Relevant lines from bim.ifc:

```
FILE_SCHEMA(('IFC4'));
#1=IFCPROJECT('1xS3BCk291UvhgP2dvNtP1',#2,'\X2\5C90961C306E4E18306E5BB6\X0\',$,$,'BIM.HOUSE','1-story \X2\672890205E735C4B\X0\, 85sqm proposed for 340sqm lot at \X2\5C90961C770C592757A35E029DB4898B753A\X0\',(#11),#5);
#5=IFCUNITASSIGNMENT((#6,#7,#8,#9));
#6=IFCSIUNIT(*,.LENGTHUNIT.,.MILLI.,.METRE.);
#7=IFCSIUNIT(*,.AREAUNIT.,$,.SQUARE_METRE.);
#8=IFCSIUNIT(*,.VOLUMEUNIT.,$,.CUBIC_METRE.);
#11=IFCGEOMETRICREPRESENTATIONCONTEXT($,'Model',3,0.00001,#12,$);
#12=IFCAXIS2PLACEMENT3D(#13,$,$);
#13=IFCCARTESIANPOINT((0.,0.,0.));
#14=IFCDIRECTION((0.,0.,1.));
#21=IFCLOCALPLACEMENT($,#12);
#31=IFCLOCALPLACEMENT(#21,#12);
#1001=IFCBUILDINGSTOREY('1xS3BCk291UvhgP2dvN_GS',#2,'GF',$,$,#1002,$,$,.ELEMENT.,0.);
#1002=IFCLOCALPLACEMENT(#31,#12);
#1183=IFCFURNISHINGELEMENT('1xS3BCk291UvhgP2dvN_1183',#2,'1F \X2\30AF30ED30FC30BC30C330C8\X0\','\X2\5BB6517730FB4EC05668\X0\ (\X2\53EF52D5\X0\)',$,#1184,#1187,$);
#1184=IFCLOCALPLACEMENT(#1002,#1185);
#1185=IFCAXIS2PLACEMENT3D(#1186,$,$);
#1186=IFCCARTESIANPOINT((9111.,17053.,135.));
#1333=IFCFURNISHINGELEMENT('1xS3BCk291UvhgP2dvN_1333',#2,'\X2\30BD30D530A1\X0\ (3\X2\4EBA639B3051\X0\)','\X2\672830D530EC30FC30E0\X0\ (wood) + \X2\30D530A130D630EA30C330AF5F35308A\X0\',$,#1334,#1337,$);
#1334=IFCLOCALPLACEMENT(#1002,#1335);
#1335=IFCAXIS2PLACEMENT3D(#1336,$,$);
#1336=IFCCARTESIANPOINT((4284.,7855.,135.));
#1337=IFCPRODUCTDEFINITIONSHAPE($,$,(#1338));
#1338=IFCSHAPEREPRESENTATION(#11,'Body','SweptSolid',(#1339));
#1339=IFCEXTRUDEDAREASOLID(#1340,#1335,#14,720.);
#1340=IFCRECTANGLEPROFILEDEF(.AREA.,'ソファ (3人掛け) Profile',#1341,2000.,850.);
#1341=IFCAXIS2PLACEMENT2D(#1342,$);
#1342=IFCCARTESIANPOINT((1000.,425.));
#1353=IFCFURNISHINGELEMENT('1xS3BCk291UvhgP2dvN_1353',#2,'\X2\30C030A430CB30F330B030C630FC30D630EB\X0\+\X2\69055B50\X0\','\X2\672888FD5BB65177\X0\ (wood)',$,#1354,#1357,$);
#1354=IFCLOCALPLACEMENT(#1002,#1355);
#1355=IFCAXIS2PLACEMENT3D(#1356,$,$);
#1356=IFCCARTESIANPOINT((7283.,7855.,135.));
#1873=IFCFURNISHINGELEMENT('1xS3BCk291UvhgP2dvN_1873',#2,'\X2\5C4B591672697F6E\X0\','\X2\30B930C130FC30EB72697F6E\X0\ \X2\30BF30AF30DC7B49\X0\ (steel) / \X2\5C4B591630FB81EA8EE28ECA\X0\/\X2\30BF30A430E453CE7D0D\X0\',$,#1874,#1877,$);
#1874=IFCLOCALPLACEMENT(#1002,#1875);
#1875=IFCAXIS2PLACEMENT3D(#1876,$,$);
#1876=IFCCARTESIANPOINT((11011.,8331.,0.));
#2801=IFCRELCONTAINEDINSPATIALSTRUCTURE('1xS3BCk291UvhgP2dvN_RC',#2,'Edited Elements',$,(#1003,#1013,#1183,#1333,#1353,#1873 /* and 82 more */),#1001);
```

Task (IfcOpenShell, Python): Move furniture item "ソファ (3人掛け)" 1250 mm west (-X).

```python
import ifcopenshell
import ifcopenshell.api.geometry
import ifcopenshell.util.placement
import ifcopenshell.util.unit

model = ifcopenshell.open("bim.ifc")
unit_scale = ifcopenshell.util.unit.calculate_unit_scale(model)

item = model.by_guid("1xS3BCk291UvhgP2dvN_1333")
matrix = ifcopenshell.util.placement.get_local_placement(item.ObjectPlacement)
matrix[0, 3] -= 1.25 / unit_scale
ifcopenshell.api.geometry.edit_object_placement(model, product=item, matrix=matrix, is_si=False)

print(ifcopenshell.util.placement.get_local_placement(item.ObjectPlacement).round(3) + 0.0)

model.write("bim_edited.ifc")
```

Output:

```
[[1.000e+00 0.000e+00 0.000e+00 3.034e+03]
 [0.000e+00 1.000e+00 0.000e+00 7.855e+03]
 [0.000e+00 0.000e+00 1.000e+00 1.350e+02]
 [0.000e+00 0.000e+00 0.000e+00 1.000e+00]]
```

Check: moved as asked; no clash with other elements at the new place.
